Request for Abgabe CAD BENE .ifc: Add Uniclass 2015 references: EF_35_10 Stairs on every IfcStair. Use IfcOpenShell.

First a look at what the model holds.

```python
import ifcopenshell

model = ifcopenshell.open("Abgabe CAD BENE .ifc")
print(model.schema)
print("classifications:", [c.Name for c in model.by_type("IfcClassification")])
for ifc_class in ("IfcDoor", "IfcRoof", "IfcStair", "IfcWall", "IfcWindow"):
    print(ifc_class, len(model.by_type(ifc_class)))
```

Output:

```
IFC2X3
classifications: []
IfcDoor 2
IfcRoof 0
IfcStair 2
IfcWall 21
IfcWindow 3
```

```python
import ifcopenshell
import ifcopenshell.api.classification

model = ifcopenshell.open("Abgabe CAD BENE .ifc")

# IFC2X3 requires Source and Edition and has no link from the project to the system.
system = model.create_entity("IfcClassification", Source="NBS", Edition="2015", Name="Uniclass 2015")

codes = {
    "IfcStair": ("EF_35_10", "Stairs"),
}
for ifc_class, (code, name) in codes.items():
    products = model.by_type(ifc_class)
    ifcopenshell.api.classification.add_reference(
        model, products=products, classification=system, identification=code, name=name
    )
    print(code, len(products))

model.write("Abgabe CAD BENE _edited.ifc")
```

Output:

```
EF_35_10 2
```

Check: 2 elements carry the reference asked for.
